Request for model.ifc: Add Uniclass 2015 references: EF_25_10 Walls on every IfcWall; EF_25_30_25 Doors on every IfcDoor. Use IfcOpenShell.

First a look at what the model holds.

```python
import ifcopenshell

model = ifcopenshell.open("model.ifc")
print(model.schema)
print("classifications:", [c.Name for c in model.by_type("IfcClassification")])
for ifc_class in ("IfcDoor", "IfcRoof", "IfcStair", "IfcWall", "IfcWindow"):
    print(ifc_class, len(model.by_type(ifc_class)))
```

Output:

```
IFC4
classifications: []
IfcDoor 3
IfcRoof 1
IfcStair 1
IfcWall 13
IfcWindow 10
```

```python
import ifcopenshell
import ifcopenshell.api.classification

model = ifcopenshell.open("model.ifc")

system = ifcopenshell.api.classification.add_classification(model, classification="Uniclass 2015")

codes = {
    "IfcWall": ("EF_25_10", "Walls"),
    "IfcDoor": ("EF_25_30_25", "Doors"),
}
for ifc_class, (code, name) in codes.items():
    products = model.by_type(ifc_class)
    ifcopenshell.api.classification.add_reference(
        model, products=products, classification=system, identification=code, name=name
    )
    print(code, len(products))

model.write("model_edited.ifc")
```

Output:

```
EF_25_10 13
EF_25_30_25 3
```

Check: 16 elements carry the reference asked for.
